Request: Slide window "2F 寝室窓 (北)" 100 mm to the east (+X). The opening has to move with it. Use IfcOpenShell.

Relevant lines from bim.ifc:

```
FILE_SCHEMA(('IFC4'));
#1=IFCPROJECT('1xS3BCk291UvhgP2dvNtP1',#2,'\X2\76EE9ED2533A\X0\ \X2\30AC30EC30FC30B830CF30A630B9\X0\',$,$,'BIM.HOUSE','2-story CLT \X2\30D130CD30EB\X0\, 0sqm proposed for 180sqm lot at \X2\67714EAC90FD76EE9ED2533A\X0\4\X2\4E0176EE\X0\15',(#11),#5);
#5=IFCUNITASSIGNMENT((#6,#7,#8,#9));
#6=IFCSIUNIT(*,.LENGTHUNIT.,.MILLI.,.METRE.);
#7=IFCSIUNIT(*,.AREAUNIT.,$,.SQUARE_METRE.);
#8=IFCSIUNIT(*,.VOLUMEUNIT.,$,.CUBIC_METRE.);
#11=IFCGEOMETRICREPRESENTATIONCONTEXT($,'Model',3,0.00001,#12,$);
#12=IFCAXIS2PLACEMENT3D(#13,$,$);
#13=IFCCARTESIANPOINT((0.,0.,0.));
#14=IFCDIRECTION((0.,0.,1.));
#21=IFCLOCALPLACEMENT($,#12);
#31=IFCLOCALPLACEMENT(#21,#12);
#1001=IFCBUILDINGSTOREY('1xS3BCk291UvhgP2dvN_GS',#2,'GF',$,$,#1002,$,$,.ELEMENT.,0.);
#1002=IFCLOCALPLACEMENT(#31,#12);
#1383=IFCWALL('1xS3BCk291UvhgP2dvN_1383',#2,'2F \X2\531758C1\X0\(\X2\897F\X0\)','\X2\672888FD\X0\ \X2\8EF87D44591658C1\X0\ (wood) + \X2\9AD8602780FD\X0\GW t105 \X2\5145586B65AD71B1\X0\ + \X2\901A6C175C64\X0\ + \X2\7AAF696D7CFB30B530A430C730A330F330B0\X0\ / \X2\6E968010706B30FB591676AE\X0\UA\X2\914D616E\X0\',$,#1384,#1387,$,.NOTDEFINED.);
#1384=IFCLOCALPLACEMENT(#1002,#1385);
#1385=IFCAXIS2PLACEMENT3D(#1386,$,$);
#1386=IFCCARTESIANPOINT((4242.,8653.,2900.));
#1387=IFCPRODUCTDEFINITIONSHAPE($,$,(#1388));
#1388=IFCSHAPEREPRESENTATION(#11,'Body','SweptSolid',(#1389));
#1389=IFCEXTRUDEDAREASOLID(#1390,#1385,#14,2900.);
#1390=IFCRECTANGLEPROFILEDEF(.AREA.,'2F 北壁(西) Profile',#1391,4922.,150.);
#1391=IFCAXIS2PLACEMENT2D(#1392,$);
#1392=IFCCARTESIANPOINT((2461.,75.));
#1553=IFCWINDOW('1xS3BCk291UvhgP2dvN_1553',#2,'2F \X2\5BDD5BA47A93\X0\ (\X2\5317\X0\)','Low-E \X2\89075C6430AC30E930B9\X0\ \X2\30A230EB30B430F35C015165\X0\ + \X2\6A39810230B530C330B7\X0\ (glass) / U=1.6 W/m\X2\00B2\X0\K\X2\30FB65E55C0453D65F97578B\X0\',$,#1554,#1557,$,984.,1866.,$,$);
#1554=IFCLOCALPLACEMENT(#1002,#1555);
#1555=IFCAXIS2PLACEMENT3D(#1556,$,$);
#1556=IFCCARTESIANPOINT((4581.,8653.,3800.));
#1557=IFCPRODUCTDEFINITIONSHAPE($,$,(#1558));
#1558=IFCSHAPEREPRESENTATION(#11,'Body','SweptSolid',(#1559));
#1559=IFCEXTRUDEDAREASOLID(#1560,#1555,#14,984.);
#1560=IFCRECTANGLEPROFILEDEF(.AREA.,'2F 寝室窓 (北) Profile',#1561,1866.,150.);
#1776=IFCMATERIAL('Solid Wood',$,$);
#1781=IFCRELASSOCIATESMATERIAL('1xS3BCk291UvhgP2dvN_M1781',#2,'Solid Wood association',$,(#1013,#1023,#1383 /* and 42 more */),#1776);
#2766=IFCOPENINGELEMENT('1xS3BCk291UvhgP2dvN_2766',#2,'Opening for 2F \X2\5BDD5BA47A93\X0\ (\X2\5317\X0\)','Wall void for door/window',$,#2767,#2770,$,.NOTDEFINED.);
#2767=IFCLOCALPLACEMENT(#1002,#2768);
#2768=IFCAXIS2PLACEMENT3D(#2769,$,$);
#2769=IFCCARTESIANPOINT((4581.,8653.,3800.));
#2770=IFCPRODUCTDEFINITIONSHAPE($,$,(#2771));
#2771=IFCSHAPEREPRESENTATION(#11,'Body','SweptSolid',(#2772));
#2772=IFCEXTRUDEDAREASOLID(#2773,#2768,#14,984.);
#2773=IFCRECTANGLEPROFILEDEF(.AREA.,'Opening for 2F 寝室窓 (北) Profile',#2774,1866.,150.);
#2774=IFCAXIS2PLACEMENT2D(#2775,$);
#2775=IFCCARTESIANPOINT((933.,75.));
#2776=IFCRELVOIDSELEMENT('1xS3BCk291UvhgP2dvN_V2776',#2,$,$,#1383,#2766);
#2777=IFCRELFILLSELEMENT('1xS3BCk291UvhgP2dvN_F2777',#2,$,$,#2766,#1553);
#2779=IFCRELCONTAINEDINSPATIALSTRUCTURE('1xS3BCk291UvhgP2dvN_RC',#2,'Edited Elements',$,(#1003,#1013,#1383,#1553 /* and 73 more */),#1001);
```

```python
import ifcopenshell
import ifcopenshell.api.geometry
import ifcopenshell.util.placement
import ifcopenshell.util.unit

model = ifcopenshell.open("bim.ifc")
unit_scale = ifcopenshell.util.unit.calculate_unit_scale(model)

window = model.by_guid("1xS3BCk291UvhgP2dvN_1553")
opening = window.FillsVoids[0].RelatingOpeningElement
wall = opening.VoidsElements[0].RelatingBuildingElement

wall_matrix = ifcopenshell.util.placement.get_local_placement(wall.ObjectPlacement)
shift = wall_matrix[:3, 0] * 0.1 / unit_scale
before = ifcopenshell.util.placement.get_local_placement(window.ObjectPlacement)[:3, 3].copy()

# The window is not placed relative to its opening, so move both.
for product in (opening, window):
    matrix = ifcopenshell.util.placement.get_local_placement(product.ObjectPlacement)
    matrix[:3, 3] += shift
    ifcopenshell.api.geometry.edit_object_placement(model, product=product, matrix=matrix, is_si=False)

after = ifcopenshell.util.placement.get_local_placement(window.ObjectPlacement)[:3, 3]
print("window moved by", (after - before).round(3) + 0.0)

model.write("bim_rev.ifc")
```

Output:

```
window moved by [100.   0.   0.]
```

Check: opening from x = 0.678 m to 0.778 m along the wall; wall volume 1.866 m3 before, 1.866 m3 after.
